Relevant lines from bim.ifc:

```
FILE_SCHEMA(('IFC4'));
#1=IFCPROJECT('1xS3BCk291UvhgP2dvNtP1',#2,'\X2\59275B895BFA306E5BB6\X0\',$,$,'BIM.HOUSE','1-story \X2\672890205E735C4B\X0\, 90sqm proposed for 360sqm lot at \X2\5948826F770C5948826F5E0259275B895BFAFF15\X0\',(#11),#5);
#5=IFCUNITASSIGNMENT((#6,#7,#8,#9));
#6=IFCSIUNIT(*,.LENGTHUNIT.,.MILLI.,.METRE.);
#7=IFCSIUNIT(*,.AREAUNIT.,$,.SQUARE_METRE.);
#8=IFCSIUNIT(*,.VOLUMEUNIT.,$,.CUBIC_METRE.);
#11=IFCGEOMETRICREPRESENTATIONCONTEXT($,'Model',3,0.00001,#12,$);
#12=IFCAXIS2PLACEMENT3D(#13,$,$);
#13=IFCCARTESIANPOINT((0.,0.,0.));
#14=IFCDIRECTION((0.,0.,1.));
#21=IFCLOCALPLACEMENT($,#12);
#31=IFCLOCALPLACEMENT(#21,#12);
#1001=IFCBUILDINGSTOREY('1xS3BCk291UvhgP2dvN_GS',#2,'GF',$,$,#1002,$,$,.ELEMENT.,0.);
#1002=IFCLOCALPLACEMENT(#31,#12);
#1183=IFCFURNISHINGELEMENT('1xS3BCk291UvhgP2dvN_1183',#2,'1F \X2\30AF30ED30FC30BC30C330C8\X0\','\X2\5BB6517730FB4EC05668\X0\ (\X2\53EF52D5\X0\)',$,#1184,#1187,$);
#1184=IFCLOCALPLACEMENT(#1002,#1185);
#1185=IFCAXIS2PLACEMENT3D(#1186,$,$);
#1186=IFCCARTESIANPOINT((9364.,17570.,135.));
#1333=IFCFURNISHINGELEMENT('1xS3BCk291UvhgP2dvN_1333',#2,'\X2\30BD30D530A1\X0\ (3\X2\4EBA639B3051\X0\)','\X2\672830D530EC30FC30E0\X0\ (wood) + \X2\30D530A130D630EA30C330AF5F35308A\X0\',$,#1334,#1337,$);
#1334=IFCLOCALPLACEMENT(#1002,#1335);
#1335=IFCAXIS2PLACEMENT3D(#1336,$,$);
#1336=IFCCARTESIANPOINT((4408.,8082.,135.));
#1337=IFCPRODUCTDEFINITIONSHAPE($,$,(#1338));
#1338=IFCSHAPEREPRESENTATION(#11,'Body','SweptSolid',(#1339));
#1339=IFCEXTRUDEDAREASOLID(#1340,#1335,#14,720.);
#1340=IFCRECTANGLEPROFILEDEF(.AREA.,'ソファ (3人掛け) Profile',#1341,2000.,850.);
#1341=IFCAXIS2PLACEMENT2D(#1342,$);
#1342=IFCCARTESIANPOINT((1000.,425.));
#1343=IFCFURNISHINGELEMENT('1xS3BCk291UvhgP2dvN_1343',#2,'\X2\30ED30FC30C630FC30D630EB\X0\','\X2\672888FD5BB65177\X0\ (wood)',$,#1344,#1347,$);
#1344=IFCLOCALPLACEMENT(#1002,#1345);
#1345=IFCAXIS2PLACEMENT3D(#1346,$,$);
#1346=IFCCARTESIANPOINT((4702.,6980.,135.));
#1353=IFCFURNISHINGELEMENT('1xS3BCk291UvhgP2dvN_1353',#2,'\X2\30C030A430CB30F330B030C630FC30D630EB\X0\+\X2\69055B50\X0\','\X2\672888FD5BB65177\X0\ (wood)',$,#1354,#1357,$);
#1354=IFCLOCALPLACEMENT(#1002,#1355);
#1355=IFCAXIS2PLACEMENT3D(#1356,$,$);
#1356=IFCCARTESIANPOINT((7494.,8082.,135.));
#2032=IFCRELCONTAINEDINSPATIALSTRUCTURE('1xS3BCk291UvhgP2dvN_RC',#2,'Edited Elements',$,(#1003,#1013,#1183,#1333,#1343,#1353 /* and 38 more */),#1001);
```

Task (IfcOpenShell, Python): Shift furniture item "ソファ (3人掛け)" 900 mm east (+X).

```python
import ifcopenshell
import ifcopenshell.api.geometry
import ifcopenshell.util.placement

model = ifcopenshell.open("bim.ifc")

item = model.by_guid("1xS3BCk291UvhgP2dvN_1333")
matrix = ifcopenshell.util.placement.get_local_placement(item.ObjectPlacement)
matrix[0, 3] += 900.0
ifcopenshell.api.geometry.edit_object_placement(model, product=item, matrix=matrix, is_si=False)

print(ifcopenshell.util.placement.get_local_placement(item.ObjectPlacement).round(3) + 0.0)

model.write("bim_v2.ifc")
```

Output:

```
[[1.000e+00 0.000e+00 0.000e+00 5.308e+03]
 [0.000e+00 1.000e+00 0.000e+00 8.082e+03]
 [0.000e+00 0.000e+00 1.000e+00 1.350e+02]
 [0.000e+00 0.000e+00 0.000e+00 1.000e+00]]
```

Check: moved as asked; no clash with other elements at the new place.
